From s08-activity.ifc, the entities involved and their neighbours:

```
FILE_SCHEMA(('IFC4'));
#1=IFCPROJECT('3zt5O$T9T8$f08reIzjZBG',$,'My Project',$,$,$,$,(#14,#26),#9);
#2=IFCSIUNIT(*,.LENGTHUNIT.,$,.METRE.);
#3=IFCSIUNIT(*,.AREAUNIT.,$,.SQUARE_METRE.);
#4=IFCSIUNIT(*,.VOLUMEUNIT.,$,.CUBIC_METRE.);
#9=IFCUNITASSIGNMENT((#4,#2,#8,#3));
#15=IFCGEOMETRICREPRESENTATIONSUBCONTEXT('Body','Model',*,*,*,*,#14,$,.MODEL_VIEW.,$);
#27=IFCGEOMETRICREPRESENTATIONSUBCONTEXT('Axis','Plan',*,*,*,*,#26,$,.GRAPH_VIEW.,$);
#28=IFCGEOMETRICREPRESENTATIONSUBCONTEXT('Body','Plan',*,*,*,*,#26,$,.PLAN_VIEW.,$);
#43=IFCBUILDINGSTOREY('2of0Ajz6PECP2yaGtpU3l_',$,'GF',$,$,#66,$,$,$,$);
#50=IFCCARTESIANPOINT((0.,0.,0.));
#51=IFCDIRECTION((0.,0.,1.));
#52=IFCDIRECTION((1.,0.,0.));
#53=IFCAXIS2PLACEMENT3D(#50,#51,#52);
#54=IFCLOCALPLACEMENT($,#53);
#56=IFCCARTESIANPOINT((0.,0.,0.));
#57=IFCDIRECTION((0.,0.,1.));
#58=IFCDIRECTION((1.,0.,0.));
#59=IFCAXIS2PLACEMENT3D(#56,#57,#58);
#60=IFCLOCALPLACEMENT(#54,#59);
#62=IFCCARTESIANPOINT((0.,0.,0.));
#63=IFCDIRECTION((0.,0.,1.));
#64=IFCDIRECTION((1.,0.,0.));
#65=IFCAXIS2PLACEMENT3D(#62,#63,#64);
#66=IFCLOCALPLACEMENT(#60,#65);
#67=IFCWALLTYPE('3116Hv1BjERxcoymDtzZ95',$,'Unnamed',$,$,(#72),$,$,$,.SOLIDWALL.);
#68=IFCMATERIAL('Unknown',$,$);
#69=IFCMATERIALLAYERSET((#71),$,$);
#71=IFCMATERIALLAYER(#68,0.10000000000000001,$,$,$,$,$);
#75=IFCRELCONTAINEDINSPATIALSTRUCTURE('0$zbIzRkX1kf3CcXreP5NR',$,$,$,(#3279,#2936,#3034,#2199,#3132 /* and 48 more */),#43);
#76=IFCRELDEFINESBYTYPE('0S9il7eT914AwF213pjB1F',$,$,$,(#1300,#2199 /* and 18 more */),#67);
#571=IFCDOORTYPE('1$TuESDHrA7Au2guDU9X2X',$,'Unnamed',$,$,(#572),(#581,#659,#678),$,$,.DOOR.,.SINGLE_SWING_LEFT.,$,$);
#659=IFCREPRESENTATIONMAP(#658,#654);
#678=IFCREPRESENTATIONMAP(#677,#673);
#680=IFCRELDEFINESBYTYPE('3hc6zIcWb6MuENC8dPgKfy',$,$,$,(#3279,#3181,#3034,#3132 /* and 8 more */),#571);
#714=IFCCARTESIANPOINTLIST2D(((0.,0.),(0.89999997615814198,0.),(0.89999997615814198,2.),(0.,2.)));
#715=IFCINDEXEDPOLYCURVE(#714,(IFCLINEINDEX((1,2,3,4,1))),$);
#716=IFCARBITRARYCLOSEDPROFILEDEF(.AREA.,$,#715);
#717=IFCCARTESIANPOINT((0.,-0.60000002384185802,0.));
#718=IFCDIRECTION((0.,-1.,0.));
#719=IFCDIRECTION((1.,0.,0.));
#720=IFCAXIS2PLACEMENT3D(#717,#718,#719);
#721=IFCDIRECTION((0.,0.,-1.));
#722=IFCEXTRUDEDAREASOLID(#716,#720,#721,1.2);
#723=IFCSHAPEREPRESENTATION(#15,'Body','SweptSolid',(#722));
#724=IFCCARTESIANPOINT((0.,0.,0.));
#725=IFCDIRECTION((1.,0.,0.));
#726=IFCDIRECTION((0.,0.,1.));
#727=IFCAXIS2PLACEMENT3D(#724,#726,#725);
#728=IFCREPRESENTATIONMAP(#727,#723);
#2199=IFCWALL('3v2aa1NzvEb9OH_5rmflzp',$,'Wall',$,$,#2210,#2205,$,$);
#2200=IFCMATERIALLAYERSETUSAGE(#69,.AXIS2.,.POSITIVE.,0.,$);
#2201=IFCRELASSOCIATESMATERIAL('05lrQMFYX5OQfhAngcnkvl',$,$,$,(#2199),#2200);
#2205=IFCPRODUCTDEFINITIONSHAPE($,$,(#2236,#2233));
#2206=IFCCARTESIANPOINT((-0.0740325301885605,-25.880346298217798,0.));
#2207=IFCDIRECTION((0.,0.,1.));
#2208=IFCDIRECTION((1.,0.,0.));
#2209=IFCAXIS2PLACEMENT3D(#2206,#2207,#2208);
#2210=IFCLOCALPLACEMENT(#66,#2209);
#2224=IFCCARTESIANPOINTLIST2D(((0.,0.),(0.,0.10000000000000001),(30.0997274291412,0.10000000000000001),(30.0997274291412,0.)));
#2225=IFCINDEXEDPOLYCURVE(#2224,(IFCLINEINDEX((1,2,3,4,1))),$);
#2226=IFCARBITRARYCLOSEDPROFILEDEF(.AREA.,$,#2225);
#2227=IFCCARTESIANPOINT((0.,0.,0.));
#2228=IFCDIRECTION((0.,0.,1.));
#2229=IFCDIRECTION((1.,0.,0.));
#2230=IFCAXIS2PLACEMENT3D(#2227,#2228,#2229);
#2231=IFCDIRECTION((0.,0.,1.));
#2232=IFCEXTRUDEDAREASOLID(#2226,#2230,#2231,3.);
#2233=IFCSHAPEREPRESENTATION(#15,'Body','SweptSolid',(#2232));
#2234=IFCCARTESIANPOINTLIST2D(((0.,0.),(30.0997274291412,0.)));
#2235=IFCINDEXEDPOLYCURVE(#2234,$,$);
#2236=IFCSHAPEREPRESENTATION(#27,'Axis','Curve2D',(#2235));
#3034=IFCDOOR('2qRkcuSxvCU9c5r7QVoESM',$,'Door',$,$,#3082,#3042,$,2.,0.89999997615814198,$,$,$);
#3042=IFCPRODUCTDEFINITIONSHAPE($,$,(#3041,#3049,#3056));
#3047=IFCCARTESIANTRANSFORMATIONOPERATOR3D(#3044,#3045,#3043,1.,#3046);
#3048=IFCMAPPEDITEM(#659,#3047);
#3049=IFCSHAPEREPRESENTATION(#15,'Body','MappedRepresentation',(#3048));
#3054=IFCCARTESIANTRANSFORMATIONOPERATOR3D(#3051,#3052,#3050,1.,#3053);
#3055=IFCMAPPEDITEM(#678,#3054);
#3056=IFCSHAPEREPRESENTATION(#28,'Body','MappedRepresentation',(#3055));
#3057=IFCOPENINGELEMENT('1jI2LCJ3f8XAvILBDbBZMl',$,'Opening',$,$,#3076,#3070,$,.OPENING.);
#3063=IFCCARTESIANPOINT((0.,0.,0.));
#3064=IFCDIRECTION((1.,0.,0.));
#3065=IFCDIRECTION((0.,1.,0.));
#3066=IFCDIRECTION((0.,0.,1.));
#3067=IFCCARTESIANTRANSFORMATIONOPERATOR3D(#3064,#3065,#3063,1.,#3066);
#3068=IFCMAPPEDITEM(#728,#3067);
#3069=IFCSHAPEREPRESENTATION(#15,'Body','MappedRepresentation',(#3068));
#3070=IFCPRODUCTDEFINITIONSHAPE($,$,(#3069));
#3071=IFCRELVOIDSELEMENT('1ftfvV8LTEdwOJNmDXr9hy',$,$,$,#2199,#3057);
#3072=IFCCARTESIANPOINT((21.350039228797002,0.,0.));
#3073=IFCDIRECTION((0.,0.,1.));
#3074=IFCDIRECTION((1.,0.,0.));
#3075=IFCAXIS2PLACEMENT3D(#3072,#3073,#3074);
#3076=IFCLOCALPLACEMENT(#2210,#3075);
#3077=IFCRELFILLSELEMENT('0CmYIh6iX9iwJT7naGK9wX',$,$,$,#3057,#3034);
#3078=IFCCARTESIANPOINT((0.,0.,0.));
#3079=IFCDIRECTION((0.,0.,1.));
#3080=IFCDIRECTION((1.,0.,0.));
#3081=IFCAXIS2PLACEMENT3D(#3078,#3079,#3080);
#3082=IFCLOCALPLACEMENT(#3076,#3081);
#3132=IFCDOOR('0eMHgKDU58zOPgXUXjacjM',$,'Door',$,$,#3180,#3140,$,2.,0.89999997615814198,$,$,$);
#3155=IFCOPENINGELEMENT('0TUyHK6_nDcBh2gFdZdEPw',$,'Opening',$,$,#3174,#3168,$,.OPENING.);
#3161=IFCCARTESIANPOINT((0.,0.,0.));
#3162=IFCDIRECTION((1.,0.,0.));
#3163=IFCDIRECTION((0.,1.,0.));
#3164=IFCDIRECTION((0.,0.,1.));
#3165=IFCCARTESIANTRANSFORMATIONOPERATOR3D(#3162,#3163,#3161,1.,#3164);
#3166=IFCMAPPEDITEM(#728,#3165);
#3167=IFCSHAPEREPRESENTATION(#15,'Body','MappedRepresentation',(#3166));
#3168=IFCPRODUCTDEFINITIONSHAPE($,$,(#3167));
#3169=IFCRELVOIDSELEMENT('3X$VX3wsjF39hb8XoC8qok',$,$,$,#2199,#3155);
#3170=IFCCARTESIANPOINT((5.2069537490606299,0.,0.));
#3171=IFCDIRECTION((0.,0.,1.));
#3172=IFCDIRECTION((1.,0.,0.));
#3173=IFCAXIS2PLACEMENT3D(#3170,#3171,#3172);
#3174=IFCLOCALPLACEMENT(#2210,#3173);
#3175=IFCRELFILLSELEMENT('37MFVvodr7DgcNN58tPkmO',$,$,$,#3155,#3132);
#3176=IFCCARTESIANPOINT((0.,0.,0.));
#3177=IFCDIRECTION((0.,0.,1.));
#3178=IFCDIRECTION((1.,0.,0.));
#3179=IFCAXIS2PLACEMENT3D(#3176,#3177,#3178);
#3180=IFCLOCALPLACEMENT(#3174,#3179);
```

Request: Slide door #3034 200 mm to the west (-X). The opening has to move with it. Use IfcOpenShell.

```python
import ifcopenshell
import ifcopenshell.api.geometry
import ifcopenshell.util.placement
import ifcopenshell.util.unit

model = ifcopenshell.open("s08-activity.ifc")
unit_scale = ifcopenshell.util.unit.calculate_unit_scale(model)

door = model.by_guid("2qRkcuSxvCU9c5r7QVoESM")
opening = door.FillsVoids[0].RelatingOpeningElement
wall = opening.VoidsElements[0].RelatingBuildingElement

wall_matrix = ifcopenshell.util.placement.get_local_placement(wall.ObjectPlacement)
shift = wall_matrix[:3, 0] * -0.2 / unit_scale
before = ifcopenshell.util.placement.get_local_placement(door.ObjectPlacement)[:3, 3].copy()

# The door is placed relative to its opening, so it follows when the opening moves.
matrix = ifcopenshell.util.placement.get_local_placement(opening.ObjectPlacement)
matrix[:3, 3] += shift
ifcopenshell.api.geometry.edit_object_placement(
    model, product=opening, matrix=matrix, is_si=False, should_transform_children=True
)

after = ifcopenshell.util.placement.get_local_placement(door.ObjectPlacement)[:3, 3]
print("door moved by", (after - before).round(3) + 0.0)

model.write("s08-activity_rev.ifc")
```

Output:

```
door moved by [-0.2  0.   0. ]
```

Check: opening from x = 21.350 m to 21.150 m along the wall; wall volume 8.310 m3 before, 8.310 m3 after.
